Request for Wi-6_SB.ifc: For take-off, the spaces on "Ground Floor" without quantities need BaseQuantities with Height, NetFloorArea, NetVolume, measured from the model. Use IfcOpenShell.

First a look at what the model holds.

```python
import ifcopenshell
import ifcopenshell.util.element
import ifcopenshell.util.unit

model = ifcopenshell.open("Wi-6_SB.ifc")
print(model.schema)
for unit_type in ("LENGTHUNIT", "AREAUNIT", "VOLUMEUNIT"):
    print(unit_type, ifcopenshell.util.unit.calculate_unit_scale(model, unit_type))
storey = next(s for s in model.by_type("IfcBuildingStorey") if s.Name == "Ground Floor")
spaces = [e for e in ifcopenshell.util.element.get_decomposition(storey) if e.is_a("IfcSpace")]
for e in sorted(spaces, key=lambda e: e.id()):
    print(e.id(), e.is_a(), e.Name, list(ifcopenshell.util.element.get_psets(e, qtos_only=True)), sep=" | ")
```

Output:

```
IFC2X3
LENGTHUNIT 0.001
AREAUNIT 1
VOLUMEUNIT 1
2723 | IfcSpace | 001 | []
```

```python
import ifcopenshell
import ifcopenshell.api.pset
import ifcopenshell.geom
import ifcopenshell.util.element
import ifcopenshell.util.shape
import ifcopenshell.util.unit

model = ifcopenshell.open("Wi-6_SB.ifc")
unit_scale = ifcopenshell.util.unit.calculate_unit_scale(model)
area_scale = ifcopenshell.util.unit.calculate_unit_scale(model, "AREAUNIT")
volume_scale = ifcopenshell.util.unit.calculate_unit_scale(model, "VOLUMEUNIT")
settings = ifcopenshell.geom.settings()

storey = next(s for s in model.by_type("IfcBuildingStorey") if s.Name == "Ground Floor")
spaces = [e for e in ifcopenshell.util.element.get_decomposition(storey) if e.is_a("IfcSpace")]

for e in sorted(spaces, key=lambda e: e.id()):
    if ifcopenshell.util.element.get_psets(e, qtos_only=True, should_inherit=False):
        continue
    # Geometry comes back in metres, in the element's own axes.
    shape = ifcopenshell.geom.create_shape(settings, e)
    values = {
        "Height": ifcopenshell.util.shape.get_z(shape.geometry) / unit_scale,
        "NetFloorArea": ifcopenshell.util.shape.get_footprint_area(shape.geometry) / area_scale,
        "NetVolume": ifcopenshell.util.shape.get_volume(shape.geometry) / volume_scale,
    }
    qto = ifcopenshell.api.pset.add_qto(model, product=e, name="BaseQuantities")
    ifcopenshell.api.pset.edit_qto(model, qto=qto, properties=values)
    print(e.id(), {k: round(v, 3) for k, v in values.items()})

model.write("Wi-6_SB_rev.ifc")
```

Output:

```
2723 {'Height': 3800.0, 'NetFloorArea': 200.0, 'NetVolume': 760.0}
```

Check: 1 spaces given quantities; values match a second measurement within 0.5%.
